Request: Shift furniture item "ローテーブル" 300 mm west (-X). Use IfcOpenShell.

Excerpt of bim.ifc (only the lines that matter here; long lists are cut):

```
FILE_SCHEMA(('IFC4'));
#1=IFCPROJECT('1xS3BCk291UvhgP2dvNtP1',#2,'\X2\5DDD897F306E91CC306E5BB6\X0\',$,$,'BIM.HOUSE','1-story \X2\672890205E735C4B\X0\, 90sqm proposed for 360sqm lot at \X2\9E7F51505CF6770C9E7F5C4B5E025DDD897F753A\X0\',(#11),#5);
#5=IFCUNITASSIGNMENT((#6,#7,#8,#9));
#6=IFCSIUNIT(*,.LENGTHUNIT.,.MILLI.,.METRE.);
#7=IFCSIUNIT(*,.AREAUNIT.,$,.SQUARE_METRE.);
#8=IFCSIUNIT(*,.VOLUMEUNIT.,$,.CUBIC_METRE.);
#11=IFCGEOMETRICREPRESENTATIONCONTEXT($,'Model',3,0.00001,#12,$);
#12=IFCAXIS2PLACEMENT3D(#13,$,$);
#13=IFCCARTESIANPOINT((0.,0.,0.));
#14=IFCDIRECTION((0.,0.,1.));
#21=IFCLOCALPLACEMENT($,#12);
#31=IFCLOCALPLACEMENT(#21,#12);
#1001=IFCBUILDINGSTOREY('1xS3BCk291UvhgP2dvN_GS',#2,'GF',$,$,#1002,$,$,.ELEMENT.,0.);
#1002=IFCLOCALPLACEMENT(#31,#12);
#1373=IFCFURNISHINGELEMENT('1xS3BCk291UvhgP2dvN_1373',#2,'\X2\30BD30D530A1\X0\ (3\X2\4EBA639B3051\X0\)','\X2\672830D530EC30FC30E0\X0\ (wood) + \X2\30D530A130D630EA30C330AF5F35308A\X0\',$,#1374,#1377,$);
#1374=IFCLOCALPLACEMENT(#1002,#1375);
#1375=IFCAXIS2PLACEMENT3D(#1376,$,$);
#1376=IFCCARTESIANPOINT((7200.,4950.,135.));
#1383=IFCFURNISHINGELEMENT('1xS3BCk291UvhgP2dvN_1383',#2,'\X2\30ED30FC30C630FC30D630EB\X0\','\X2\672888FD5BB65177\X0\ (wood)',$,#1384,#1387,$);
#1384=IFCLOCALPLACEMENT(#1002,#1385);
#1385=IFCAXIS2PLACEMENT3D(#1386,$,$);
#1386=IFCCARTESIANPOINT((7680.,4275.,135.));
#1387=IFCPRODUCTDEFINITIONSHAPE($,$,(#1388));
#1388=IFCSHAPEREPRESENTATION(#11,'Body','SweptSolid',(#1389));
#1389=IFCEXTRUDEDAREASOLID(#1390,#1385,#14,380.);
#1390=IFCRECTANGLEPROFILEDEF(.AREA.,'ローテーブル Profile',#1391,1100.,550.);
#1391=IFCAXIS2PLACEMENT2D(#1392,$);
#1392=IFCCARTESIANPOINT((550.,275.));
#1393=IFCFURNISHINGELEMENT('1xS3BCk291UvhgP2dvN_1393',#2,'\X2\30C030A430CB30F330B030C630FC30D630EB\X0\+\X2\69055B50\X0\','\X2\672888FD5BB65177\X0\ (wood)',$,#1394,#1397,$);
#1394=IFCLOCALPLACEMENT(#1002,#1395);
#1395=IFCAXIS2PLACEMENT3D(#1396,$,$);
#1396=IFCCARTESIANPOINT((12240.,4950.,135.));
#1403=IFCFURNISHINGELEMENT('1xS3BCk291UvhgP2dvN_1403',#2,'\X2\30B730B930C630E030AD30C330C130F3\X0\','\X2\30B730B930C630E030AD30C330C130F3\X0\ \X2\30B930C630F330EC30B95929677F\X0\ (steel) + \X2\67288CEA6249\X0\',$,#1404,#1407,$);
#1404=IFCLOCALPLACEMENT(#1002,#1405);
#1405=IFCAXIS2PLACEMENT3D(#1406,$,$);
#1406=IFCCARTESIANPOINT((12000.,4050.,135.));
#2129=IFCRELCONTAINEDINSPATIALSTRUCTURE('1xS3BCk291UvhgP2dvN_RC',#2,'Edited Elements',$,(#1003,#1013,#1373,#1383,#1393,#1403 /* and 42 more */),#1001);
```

```python
import ifcopenshell
import ifcopenshell.api.geometry
import ifcopenshell.util.placement

model = ifcopenshell.open("bim.ifc")

item = model.by_guid("1xS3BCk291UvhgP2dvN_1383")
matrix = ifcopenshell.util.placement.get_local_placement(item.ObjectPlacement)
matrix[0, 3] -= 300.0
ifcopenshell.api.geometry.edit_object_placement(model, product=item, matrix=matrix, is_si=False)

print(ifcopenshell.util.placement.get_local_placement(item.ObjectPlacement).round(3) + 0.0)

model.write("bim_updated.ifc")
```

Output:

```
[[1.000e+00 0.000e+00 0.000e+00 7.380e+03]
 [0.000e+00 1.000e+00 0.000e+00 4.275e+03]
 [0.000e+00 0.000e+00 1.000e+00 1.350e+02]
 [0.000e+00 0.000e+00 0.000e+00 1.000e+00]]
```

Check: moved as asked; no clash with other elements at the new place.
